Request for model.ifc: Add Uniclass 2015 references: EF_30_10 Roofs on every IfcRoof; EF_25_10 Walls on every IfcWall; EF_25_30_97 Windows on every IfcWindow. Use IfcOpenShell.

First a look at what the model holds.

```python
import ifcopenshell

model = ifcopenshell.open("model.ifc")
print(model.schema)
print("classifications:", [c.Name for c in model.by_type("IfcClassification")])
for ifc_class in ("IfcDoor", "IfcRoof", "IfcStair", "IfcWall", "IfcWindow"):
    print(ifc_class, len(model.by_type(ifc_class)))
```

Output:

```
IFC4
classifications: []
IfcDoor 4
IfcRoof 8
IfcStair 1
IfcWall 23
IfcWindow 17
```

```python
import ifcopenshell
import ifcopenshell.api.classification

model = ifcopenshell.open("model.ifc")

system = ifcopenshell.api.classification.add_classification(model, classification="Uniclass 2015")

codes = {
    "IfcRoof": ("EF_30_10", "Roofs"),
    "IfcWall": ("EF_25_10", "Walls"),
    "IfcWindow": ("EF_25_30_97", "Windows"),
}
for ifc_class, (code, name) in codes.items():
    products = model.by_type(ifc_class)
    ifcopenshell.api.classification.add_reference(
        model, products=products, classification=system, identification=code, name=name
    )
    print(code, len(products))

model.write("model_v2.ifc")
```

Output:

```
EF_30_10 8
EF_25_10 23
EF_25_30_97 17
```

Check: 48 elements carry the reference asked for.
